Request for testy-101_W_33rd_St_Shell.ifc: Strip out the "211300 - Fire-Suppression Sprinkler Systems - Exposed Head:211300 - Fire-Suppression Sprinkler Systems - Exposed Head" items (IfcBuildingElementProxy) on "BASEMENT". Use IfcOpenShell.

First a look at what the model holds.

```python
import ifcopenshell
import ifcopenshell.util.element

model = ifcopenshell.open("testy-101_W_33rd_St_Shell.ifc")
print(model.schema)
storey = next(s for s in model.by_type("IfcBuildingStorey") if s.Name == "BASEMENT")
proxies = [e for e in ifcopenshell.util.element.get_decomposition(storey) if e.is_a("IfcBuildingElementProxy")]
seen = {}
for e in proxies:
    element_type = ifcopenshell.util.element.get_type(e)
    name = element_type.Name if element_type not in (None, e) else None
    seen[name] = seen.get(name, 0) + 1
for name, count in sorted(seen.items(), key=str):
    print(count, "x", name)
```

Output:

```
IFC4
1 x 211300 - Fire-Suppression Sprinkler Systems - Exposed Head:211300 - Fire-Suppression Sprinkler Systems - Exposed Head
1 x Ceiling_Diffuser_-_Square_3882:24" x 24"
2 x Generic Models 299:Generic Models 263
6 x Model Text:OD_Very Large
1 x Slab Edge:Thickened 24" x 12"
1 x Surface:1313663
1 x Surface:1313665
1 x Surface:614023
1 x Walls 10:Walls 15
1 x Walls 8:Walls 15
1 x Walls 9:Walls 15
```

```python
import ifcopenshell
import ifcopenshell.api.root
import ifcopenshell.util.element

model = ifcopenshell.open("testy-101_W_33rd_St_Shell.ifc")

storey = next(s for s in model.by_type("IfcBuildingStorey") if s.Name == "BASEMENT")
proxies = [e for e in ifcopenshell.util.element.get_decomposition(storey) if e.is_a("IfcBuildingElementProxy")]
targets = [e for e in proxies if (t := ifcopenshell.util.element.get_type(e)) not in (None, e) and t.Name == "211300 - Fire-Suppression Sprinkler Systems - Exposed Head:211300 - Fire-Suppression Sprinkler Systems - Exposed Head"]

for e in targets:
    ifcopenshell.api.root.remove_product(model, product=e)
print(len(targets), "removed")

model.write("testy-101_W_33rd_St_Shell-out.ifc")
```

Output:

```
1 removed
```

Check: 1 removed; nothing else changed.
